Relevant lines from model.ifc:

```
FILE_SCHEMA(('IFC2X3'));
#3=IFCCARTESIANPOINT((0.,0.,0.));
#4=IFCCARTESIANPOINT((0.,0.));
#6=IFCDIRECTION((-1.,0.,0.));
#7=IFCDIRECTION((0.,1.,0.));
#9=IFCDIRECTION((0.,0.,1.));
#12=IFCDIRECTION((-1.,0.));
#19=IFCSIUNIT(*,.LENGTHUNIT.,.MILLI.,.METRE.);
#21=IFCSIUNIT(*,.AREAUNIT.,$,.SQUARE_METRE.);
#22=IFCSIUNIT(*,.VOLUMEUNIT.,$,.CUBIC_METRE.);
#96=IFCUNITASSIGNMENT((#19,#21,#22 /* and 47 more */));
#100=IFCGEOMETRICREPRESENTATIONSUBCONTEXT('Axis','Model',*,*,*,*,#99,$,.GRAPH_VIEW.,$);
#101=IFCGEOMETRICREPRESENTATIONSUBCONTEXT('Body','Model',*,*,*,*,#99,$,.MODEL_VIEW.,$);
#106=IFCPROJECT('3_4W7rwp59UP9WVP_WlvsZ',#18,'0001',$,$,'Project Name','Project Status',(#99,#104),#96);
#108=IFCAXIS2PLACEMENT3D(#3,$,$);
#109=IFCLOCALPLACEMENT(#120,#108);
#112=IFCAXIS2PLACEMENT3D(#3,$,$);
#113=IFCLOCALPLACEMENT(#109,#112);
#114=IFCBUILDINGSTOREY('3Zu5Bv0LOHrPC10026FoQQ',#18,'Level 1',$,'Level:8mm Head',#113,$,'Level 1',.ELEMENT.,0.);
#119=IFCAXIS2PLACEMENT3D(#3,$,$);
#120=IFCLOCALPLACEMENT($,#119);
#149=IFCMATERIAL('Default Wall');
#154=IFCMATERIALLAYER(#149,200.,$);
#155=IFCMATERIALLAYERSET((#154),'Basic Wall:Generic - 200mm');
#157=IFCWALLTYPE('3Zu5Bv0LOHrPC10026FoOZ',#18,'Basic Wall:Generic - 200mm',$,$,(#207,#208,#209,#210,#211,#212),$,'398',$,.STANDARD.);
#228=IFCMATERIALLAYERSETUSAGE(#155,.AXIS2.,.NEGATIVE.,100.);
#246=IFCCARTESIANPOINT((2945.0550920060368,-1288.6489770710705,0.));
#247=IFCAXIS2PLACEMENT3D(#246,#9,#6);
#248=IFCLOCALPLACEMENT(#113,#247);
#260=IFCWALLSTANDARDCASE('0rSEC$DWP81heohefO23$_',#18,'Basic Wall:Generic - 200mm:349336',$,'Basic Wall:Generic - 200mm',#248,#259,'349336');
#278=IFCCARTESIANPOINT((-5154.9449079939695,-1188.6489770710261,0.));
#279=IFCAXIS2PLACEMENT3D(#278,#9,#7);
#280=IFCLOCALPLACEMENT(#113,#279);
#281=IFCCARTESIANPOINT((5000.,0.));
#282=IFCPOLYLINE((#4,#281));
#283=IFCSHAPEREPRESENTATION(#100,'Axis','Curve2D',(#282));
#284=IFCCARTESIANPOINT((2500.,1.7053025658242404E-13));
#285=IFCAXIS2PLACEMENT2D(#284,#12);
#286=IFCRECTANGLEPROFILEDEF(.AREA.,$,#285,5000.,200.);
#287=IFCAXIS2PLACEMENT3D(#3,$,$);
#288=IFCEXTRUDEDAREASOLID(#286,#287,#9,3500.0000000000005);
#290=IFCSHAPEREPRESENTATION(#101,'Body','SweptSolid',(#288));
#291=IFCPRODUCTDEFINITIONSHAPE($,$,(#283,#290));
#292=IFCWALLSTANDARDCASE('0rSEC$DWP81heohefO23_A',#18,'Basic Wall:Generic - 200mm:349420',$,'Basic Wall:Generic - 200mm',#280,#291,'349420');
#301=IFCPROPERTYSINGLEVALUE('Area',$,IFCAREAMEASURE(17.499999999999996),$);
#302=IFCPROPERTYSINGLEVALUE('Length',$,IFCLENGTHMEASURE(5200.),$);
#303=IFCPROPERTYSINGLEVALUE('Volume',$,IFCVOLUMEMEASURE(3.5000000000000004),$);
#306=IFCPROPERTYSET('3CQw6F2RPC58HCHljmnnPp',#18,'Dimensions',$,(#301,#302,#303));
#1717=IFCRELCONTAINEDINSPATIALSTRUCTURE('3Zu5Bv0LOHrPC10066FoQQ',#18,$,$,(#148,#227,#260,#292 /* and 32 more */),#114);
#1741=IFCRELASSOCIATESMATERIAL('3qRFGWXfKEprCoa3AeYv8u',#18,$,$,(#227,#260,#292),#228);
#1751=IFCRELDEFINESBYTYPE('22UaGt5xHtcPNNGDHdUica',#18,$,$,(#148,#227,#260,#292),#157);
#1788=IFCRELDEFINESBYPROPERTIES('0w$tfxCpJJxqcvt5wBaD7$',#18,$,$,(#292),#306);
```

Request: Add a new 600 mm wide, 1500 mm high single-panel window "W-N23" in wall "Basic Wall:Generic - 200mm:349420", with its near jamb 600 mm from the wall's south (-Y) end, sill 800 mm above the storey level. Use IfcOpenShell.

```python
import numpy as np
import ifcopenshell
import ifcopenshell.api.feature
import ifcopenshell.api.geometry
import ifcopenshell.api.pset
import ifcopenshell.api.root
import ifcopenshell.api.spatial
import ifcopenshell.api.type
import ifcopenshell.geom
import ifcopenshell.util.element
import ifcopenshell.util.placement
import ifcopenshell.util.representation
import ifcopenshell.util.shape
import ifcopenshell.util.unit

model = ifcopenshell.open("model.ifc")
unit_scale = ifcopenshell.util.unit.calculate_unit_scale(model)
area_scale = ifcopenshell.util.unit.calculate_unit_scale(model, "AREAUNIT")
volume_scale = ifcopenshell.util.unit.calculate_unit_scale(model, "VOLUMEUNIT")
settings = ifcopenshell.geom.settings()


def volume(element):
    """Net volume in cubic metres, openings subtracted."""
    shape = ifcopenshell.geom.create_shape(settings, element)
    return ifcopenshell.util.shape.get_volume(shape.geometry)


wall = model.by_guid("0rSEC$DWP81heohefO23_A")
storey = ifcopenshell.util.element.get_container(wall, ifc_class="IfcBuildingStorey")
context = ifcopenshell.util.representation.get_context(model, "Model", "Body", "MODEL_VIEW")
before = volume(wall)

width, height, from_end, sill = 0.6, 1.5, 0.6, 0.8  # metres

# The wall runs along its own X axis, and the end named is its -X end.
wall_shape = ifcopenshell.geom.create_shape(settings, wall)
x, y, z = ifcopenshell.util.shape.get_vertices(wall_shape.geometry).T
start = x.min() + from_end
face, thickness = float(y.min()), float(y.max() - y.min())
wall_matrix = ifcopenshell.util.placement.get_local_placement(wall.ObjectPlacement)
level = ifcopenshell.util.placement.get_local_placement(storey.ObjectPlacement)[2, 3]


def in_wall(x, y):
    """Placement at x, y metres in the wall's axes, at sill height."""
    matrix = wall_matrix.copy()
    matrix[:, 3] = wall_matrix @ np.array([x / unit_scale, y / unit_scale, 0.0, 1.0])
    matrix[2, 3] = level + sill / unit_scale
    return matrix


# Opening: a box that overshoots both wall faces by 50 mm.
opening = ifcopenshell.api.root.create_entity(model, ifc_class="IfcOpeningElement")
box = ifcopenshell.api.geometry.add_wall_representation(
    model, context=context, length=width, height=height, thickness=thickness + 0.1
)
ifcopenshell.api.geometry.assign_representation(model, product=opening, representation=box)
ifcopenshell.api.geometry.edit_object_placement(model, product=opening, matrix=in_wall(start, face - 0.05), is_si=False)
ifcopenshell.api.feature.add_feature(model, feature=opening, element=wall)

window = ifcopenshell.api.root.create_entity(model, ifc_class="IfcWindow", name="W-N23")
window.OverallWidth, window.OverallHeight = width / unit_scale, height / unit_scale
body = ifcopenshell.api.geometry.add_window_representation(
    model,
    context=context,
    overall_width=window.OverallWidth,
    overall_height=window.OverallHeight,
    partition_type="SINGLE_PANEL",
)
ifcopenshell.api.geometry.assign_representation(model, product=window, representation=body)
ifcopenshell.api.spatial.assign_container(model, products=[window], relating_structure=storey)
fills = ifcopenshell.api.feature.add_filling(model, opening=opening, element=window)
fills.OwnerHistory = window.OwnerHistory  # required in IFC2X3

# IFC2X3 keeps the operation on the window style.
style = ifcopenshell.api.root.create_entity(model, ifc_class="IfcWindowStyle", name="W-N23")
style.OperationType, style.ConstructionType = "SINGLE_PANEL", "NOTDEFINED"
style.ParameterTakesPrecedence = style.Sizeable = False
ifcopenshell.api.type.assign_type(model, related_objects=[window], relating_type=style)

# Centre the window in the wall's thickness.
ifcopenshell.api.geometry.edit_object_placement(model, product=window, matrix=in_wall(start, face), is_si=False)
window_shape = ifcopenshell.geom.create_shape(settings, window)
depth = ifcopenshell.util.shape.get_vertices(window_shape.geometry)[:, 1]
offset = face + thickness / 2 - (depth.min() + depth.max()) / 2
ifcopenshell.api.geometry.edit_object_placement(model, product=window, matrix=in_wall(start, offset), is_si=False)

after = volume(wall)

# Update the wall's stored quantities.
pset = model.by_id(ifcopenshell.util.element.get_pset(wall, "Dimensions", should_inherit=False)["id"])
ifcopenshell.api.pset.edit_pset(model, pset=pset, properties={
    "Area": model.create_entity("IfcAreaMeasure", after / thickness / area_scale),
    "Volume": model.create_entity("IfcVolumeMeasure", after / volume_scale),
})

print(f"wall volume {before:.3f} -> {after:.3f} m3")

model.write("model_updated.ifc")
```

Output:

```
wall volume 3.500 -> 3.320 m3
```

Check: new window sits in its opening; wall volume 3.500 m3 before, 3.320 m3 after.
